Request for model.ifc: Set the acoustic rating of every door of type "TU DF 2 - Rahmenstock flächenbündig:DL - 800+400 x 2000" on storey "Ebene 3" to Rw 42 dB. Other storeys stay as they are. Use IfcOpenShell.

First a look at what the model holds.

```python
import ifcopenshell
import ifcopenshell.util.element

model = ifcopenshell.open("model.ifc")
print(model.schema)
storey = next(s for s in model.by_type("IfcBuildingStorey") if s.Name == "Ebene 3")
doors = [e for e in ifcopenshell.util.element.get_decomposition(storey) if e.is_a("IfcDoor")]
seen = {}
for e in doors:
    element_type = ifcopenshell.util.element.get_type(e)
    key = (element_type.Name if element_type != e and element_type else None, ifcopenshell.util.element.get_pset(e, "Pset_DoorCommon", "AcousticRating"))
    seen[key] = seen.get(key, 0) + 1
for (name, value), count in sorted(seen.items(), key=str):
    print(count, "x", name, "|", value)
```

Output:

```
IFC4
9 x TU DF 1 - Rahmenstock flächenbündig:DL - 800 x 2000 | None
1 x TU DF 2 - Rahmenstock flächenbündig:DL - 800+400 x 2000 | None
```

```python
import ifcopenshell
import ifcopenshell.api.pset
import ifcopenshell.util.element

model = ifcopenshell.open("model.ifc")

storey = next(s for s in model.by_type("IfcBuildingStorey") if s.Name == "Ebene 3")
doors = [e for e in ifcopenshell.util.element.get_decomposition(storey) if e.is_a("IfcDoor")]

count = 0
for e in doors:
    element_type = ifcopenshell.util.element.get_type(e)
    if element_type in (None, e) or element_type.Name != "TU DF 2 - Rahmenstock flächenbündig:DL - 800+400 x 2000":
        continue
    # add_pset returns the element's existing set when there is one.
    pset = ifcopenshell.api.pset.add_pset(model, product=e, name="Pset_DoorCommon")
    ifcopenshell.api.pset.edit_pset(model, pset=pset, properties={"AcousticRating": "Rw 42 dB"})
    count += 1

print(count, "doors updated")

model.write("model-out.ifc")
```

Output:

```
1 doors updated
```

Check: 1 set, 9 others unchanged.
